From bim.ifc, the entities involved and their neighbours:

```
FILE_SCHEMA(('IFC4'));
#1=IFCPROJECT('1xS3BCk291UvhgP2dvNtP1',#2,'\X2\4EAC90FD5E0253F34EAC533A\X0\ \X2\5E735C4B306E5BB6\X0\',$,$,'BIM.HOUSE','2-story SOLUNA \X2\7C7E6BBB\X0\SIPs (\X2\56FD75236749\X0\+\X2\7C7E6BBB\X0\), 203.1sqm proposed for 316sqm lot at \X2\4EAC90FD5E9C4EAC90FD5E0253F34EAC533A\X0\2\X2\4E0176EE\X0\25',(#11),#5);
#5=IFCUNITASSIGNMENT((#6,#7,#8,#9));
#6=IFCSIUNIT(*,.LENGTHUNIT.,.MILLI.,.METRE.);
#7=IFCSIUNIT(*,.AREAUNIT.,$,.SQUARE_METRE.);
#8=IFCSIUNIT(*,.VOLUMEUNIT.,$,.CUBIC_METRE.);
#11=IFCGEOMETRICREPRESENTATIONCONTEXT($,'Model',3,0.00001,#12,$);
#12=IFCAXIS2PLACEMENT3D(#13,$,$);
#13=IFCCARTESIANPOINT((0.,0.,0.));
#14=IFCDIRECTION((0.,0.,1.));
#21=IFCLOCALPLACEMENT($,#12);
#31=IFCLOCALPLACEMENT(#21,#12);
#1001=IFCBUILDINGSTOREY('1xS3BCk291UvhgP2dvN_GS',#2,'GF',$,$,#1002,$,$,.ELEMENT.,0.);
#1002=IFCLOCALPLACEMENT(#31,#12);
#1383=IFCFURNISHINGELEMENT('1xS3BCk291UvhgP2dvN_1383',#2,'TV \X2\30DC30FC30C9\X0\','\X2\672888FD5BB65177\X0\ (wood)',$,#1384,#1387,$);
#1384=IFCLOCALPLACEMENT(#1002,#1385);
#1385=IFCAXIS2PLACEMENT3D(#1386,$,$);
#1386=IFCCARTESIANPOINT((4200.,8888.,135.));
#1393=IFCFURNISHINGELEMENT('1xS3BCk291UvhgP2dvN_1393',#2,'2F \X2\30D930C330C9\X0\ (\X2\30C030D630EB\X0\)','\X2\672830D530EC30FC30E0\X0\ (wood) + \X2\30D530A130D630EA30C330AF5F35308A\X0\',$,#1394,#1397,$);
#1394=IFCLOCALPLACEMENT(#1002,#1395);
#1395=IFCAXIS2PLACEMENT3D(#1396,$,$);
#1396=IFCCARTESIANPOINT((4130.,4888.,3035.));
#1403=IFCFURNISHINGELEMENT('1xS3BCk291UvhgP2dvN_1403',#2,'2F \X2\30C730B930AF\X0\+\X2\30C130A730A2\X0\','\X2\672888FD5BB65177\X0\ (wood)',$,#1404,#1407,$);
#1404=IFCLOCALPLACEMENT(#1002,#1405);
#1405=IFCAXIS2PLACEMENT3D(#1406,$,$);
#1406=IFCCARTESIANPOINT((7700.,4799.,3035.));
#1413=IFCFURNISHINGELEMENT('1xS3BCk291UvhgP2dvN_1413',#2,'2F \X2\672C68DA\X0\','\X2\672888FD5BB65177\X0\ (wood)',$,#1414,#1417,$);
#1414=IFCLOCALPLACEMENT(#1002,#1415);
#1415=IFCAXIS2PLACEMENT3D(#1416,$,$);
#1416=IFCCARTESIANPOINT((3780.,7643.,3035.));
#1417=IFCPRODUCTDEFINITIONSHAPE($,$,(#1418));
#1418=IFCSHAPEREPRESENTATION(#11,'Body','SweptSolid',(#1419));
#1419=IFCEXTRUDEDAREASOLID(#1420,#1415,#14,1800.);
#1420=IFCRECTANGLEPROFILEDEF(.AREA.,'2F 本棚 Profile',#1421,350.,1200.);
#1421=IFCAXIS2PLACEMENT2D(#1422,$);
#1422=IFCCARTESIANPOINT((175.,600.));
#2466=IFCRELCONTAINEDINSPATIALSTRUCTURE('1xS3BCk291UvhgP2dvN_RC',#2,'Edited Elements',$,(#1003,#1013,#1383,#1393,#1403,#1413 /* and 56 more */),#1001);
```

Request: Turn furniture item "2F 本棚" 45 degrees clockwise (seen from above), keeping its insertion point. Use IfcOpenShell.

```python
import ifcopenshell
import ifcopenshell.api.geometry
import ifcopenshell.util.placement

model = ifcopenshell.open("bim.ifc")

item = model.by_id(1413)
matrix = ifcopenshell.util.placement.get_local_placement(item.ObjectPlacement)
matrix = matrix @ ifcopenshell.util.placement.rotation(-45, "Z")
ifcopenshell.api.geometry.edit_object_placement(model, product=item, matrix=matrix, is_si=False)

print(ifcopenshell.util.placement.get_local_placement(item.ObjectPlacement).round(3) + 0.0)

model.write("bim_updated.ifc")
```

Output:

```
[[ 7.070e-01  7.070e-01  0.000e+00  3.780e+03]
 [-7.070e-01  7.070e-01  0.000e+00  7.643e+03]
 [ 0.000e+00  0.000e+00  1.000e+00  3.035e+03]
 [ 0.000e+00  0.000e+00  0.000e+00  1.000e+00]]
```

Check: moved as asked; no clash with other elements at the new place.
